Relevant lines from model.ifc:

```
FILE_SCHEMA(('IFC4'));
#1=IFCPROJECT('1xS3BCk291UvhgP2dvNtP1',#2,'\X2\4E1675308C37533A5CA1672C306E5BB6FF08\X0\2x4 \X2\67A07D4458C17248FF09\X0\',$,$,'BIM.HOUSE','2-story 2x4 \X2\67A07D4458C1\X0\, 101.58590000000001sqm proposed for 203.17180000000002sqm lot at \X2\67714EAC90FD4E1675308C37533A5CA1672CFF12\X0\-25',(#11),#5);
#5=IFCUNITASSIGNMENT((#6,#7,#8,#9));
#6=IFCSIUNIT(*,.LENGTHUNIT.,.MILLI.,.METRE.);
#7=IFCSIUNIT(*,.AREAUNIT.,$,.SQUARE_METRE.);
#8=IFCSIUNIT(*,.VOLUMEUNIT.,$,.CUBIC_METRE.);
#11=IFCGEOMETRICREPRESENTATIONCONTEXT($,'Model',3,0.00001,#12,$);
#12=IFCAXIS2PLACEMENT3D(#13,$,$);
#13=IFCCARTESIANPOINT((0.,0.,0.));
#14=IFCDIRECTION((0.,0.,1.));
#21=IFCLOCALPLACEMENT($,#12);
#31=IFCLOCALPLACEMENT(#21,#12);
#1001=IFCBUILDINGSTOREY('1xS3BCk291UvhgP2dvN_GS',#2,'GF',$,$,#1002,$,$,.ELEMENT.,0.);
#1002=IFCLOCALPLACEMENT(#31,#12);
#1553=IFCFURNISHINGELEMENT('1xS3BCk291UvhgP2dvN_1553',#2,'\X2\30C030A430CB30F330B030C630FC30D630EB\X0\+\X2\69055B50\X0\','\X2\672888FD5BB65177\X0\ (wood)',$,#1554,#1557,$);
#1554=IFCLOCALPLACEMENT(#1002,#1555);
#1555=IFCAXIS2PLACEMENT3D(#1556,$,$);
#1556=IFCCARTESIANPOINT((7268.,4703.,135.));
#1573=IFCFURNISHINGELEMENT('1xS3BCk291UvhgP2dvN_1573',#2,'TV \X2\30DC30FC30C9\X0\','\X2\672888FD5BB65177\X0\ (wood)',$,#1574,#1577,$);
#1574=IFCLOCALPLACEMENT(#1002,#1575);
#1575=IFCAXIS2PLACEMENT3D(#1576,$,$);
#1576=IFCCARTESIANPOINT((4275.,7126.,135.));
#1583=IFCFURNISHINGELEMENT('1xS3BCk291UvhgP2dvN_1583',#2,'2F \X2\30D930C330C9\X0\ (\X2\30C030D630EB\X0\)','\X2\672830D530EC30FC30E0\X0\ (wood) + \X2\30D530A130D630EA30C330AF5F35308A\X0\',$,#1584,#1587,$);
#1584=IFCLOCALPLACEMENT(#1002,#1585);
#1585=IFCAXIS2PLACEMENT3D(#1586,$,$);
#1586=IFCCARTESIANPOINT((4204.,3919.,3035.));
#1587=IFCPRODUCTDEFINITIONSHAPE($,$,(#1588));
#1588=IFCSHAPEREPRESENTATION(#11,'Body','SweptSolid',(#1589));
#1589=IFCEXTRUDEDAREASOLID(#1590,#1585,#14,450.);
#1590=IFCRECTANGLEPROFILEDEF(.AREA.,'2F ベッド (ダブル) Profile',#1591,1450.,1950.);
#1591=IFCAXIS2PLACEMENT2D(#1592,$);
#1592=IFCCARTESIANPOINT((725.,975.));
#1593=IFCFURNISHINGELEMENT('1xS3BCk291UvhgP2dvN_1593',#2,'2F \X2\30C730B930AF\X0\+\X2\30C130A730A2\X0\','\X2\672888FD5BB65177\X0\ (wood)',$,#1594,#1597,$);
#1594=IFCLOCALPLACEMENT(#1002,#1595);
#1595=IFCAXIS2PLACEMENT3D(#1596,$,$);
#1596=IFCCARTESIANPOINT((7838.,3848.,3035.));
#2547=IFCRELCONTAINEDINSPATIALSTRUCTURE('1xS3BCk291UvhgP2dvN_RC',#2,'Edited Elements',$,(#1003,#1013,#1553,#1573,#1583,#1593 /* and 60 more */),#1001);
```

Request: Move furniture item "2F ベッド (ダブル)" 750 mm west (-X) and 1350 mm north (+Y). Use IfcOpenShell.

```python
import ifcopenshell
import ifcopenshell.api.geometry
import ifcopenshell.util.placement

model = ifcopenshell.open("model.ifc")

item = model.by_guid("1xS3BCk291UvhgP2dvN_1583")
matrix = ifcopenshell.util.placement.get_local_placement(item.ObjectPlacement)
matrix[0, 3] -= 750.0
matrix[1, 3] += 1350.0
ifcopenshell.api.geometry.edit_object_placement(model, product=item, matrix=matrix, is_si=False)

print(ifcopenshell.util.placement.get_local_placement(item.ObjectPlacement).round(3) + 0.0)

model.write("model-out.ifc")
```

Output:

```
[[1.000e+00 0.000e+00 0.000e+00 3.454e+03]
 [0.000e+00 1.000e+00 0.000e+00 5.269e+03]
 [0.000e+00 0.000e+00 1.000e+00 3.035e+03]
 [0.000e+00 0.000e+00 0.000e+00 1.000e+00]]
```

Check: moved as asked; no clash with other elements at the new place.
